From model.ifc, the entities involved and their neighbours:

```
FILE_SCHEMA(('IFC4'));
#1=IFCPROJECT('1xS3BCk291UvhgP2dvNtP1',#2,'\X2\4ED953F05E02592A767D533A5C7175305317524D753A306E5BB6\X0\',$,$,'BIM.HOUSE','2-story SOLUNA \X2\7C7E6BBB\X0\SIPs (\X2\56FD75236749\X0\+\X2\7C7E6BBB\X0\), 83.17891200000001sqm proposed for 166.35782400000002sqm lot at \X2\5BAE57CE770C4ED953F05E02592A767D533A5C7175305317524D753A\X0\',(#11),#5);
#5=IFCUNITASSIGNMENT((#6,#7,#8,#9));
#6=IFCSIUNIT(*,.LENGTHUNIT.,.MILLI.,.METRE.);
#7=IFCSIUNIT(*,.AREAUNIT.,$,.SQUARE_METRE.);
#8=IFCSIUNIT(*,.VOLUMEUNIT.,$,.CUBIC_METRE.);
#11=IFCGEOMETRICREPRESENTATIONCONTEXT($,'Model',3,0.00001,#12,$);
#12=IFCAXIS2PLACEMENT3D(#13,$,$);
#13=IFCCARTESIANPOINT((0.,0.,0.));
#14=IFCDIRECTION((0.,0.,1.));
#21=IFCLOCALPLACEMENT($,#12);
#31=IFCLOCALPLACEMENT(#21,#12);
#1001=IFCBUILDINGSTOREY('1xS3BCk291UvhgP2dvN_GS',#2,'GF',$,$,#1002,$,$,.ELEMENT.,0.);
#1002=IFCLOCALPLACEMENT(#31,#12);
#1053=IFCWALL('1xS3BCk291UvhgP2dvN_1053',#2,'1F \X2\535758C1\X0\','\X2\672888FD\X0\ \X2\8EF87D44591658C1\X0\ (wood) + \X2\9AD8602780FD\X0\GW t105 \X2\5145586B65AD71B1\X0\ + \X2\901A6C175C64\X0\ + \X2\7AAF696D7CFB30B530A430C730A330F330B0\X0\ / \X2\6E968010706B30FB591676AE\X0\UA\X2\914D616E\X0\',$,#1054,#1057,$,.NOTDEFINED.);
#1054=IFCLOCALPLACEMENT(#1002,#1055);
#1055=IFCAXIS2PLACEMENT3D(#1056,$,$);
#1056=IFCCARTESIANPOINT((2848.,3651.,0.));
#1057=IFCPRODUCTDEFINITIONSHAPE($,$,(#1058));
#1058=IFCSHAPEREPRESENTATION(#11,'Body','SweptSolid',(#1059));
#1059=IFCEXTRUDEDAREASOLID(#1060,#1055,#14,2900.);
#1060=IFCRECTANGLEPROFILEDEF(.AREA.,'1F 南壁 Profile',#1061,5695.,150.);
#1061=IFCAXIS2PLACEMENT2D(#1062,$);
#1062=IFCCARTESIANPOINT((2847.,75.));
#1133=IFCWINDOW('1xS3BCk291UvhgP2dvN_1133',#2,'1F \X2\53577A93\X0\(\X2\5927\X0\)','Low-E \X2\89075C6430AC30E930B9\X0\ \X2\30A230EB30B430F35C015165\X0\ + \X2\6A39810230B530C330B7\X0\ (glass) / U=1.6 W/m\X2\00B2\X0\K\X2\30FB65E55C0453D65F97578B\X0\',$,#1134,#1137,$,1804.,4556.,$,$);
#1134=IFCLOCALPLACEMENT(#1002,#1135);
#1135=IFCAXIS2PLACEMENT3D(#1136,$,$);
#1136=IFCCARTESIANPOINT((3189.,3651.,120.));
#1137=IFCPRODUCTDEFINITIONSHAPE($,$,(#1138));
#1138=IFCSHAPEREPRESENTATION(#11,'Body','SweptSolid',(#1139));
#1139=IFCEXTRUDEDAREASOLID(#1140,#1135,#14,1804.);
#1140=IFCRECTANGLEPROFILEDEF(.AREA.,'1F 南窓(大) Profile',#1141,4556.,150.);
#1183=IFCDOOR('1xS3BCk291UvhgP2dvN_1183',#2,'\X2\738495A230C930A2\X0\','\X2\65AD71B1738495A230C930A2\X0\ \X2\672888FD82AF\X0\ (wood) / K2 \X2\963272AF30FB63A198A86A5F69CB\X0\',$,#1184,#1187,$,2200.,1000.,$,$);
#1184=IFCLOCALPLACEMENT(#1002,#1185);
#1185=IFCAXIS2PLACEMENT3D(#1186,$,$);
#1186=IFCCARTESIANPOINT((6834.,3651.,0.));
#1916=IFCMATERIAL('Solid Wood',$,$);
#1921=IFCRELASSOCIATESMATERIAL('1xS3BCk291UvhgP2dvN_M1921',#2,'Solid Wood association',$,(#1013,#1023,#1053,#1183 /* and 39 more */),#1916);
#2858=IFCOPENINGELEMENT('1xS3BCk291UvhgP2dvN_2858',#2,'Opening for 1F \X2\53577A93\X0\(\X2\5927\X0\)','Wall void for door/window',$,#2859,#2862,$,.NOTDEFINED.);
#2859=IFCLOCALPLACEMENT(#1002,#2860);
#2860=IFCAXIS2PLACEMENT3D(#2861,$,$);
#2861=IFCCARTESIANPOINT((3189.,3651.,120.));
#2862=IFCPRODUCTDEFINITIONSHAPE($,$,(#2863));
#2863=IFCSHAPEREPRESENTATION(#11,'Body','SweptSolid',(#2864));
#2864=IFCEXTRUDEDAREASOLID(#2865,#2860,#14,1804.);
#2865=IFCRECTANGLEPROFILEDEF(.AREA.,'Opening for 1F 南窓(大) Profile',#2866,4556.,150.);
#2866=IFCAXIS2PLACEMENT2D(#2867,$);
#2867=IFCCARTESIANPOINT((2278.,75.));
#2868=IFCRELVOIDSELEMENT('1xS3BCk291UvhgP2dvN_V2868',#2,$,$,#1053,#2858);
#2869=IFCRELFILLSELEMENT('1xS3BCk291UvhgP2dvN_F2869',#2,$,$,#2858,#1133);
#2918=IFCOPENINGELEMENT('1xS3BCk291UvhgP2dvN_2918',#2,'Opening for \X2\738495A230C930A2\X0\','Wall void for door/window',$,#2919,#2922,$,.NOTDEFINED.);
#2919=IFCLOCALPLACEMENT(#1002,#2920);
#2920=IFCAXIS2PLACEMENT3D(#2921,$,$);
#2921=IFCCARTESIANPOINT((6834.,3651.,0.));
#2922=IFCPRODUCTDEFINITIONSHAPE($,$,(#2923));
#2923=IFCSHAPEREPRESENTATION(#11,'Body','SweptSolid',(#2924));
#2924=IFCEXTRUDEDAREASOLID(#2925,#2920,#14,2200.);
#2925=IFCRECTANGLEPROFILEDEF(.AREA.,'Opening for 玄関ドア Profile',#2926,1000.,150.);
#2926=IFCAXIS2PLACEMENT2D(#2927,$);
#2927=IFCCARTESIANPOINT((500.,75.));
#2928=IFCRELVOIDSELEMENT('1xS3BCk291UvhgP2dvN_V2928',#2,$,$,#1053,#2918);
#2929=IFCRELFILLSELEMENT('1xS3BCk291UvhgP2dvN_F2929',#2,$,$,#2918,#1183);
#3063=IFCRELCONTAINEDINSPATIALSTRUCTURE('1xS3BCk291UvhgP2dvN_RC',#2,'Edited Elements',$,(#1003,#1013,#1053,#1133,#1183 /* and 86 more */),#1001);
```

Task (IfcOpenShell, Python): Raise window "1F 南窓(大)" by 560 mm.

```python
import numpy as np
import ifcopenshell
import ifcopenshell.api.geometry
import ifcopenshell.util.placement
import ifcopenshell.util.unit

model = ifcopenshell.open("model.ifc")
unit_scale = ifcopenshell.util.unit.calculate_unit_scale(model)

window = model.by_guid("1xS3BCk291UvhgP2dvN_1133")
opening = window.FillsVoids[0].RelatingOpeningElement
dz = 560.0

shift = np.array([0.0, 0.0, dz])
# The window is not placed relative to its opening, so move both.
for product in (opening, window):
    matrix = ifcopenshell.util.placement.get_local_placement(product.ObjectPlacement)
    matrix[:3, 3] += shift
    ifcopenshell.api.geometry.edit_object_placement(model, product=product, matrix=matrix, is_si=False)

print(f"moved by {dz * unit_scale:+.3f} m")

model.write("model_rev.ifc")
```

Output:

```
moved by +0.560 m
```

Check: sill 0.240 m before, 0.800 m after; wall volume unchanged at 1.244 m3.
